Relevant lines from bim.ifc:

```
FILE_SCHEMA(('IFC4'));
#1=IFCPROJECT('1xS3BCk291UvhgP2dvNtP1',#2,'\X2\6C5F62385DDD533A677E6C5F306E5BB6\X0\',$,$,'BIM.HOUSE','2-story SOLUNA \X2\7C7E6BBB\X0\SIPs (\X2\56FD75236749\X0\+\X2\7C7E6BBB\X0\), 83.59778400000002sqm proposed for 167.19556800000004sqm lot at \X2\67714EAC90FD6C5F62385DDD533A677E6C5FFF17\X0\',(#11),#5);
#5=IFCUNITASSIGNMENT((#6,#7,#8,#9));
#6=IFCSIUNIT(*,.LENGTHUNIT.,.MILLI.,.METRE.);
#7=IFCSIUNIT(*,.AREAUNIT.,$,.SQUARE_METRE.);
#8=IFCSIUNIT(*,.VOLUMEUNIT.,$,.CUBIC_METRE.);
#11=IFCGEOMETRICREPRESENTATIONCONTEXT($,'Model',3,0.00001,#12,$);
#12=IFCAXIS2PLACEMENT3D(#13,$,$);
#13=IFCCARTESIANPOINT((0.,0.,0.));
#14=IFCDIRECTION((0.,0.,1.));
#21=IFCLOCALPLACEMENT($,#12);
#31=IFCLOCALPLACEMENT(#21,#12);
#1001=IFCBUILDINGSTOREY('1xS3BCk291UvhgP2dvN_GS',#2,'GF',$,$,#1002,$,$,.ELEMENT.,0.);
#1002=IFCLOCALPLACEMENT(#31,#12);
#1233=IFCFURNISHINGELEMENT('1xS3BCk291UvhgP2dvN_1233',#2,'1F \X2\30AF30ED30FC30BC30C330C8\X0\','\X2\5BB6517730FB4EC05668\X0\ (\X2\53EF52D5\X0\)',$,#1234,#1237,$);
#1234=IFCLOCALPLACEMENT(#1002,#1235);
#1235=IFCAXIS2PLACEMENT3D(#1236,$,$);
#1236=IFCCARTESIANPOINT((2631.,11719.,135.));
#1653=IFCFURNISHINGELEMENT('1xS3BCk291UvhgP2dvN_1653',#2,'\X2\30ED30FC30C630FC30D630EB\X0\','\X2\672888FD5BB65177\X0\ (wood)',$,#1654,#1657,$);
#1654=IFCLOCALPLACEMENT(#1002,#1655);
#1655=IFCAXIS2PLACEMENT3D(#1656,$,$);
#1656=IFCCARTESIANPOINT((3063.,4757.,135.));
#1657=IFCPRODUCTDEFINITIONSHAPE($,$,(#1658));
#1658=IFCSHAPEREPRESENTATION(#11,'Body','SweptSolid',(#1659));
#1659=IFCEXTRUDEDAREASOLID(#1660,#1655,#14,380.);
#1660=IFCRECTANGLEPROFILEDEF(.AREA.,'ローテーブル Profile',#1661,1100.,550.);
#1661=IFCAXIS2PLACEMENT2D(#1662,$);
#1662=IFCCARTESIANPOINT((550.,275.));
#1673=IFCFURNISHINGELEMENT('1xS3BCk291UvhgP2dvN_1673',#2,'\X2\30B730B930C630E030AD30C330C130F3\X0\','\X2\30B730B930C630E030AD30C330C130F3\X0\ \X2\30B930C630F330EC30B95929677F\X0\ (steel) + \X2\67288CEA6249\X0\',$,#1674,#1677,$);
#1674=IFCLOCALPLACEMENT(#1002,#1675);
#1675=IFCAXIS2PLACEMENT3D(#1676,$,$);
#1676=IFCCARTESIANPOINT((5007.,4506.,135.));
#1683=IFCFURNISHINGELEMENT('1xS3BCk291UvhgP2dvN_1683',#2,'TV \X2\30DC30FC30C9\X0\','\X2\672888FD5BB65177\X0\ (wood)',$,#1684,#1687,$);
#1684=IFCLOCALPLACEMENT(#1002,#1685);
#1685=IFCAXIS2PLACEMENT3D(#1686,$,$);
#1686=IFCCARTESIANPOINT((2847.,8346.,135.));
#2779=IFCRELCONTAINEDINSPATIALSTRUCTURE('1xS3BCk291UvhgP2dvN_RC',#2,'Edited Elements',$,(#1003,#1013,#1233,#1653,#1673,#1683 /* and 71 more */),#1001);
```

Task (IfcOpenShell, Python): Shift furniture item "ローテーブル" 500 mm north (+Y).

```python
import ifcopenshell
import ifcopenshell.api.geometry
import ifcopenshell.util.placement
import ifcopenshell.util.unit

model = ifcopenshell.open("bim.ifc")
unit_scale = ifcopenshell.util.unit.calculate_unit_scale(model)

item = model.by_guid("1xS3BCk291UvhgP2dvN_1653")
matrix = ifcopenshell.util.placement.get_local_placement(item.ObjectPlacement)
matrix[1, 3] += 0.5 / unit_scale
ifcopenshell.api.geometry.edit_object_placement(model, product=item, matrix=matrix, is_si=False)

print(ifcopenshell.util.placement.get_local_placement(item.ObjectPlacement).round(3) + 0.0)

model.write("bim_updated.ifc")
```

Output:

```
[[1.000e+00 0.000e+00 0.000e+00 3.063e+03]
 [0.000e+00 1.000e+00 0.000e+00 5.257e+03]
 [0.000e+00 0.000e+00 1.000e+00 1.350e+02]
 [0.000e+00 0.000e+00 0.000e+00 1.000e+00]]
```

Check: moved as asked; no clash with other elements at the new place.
